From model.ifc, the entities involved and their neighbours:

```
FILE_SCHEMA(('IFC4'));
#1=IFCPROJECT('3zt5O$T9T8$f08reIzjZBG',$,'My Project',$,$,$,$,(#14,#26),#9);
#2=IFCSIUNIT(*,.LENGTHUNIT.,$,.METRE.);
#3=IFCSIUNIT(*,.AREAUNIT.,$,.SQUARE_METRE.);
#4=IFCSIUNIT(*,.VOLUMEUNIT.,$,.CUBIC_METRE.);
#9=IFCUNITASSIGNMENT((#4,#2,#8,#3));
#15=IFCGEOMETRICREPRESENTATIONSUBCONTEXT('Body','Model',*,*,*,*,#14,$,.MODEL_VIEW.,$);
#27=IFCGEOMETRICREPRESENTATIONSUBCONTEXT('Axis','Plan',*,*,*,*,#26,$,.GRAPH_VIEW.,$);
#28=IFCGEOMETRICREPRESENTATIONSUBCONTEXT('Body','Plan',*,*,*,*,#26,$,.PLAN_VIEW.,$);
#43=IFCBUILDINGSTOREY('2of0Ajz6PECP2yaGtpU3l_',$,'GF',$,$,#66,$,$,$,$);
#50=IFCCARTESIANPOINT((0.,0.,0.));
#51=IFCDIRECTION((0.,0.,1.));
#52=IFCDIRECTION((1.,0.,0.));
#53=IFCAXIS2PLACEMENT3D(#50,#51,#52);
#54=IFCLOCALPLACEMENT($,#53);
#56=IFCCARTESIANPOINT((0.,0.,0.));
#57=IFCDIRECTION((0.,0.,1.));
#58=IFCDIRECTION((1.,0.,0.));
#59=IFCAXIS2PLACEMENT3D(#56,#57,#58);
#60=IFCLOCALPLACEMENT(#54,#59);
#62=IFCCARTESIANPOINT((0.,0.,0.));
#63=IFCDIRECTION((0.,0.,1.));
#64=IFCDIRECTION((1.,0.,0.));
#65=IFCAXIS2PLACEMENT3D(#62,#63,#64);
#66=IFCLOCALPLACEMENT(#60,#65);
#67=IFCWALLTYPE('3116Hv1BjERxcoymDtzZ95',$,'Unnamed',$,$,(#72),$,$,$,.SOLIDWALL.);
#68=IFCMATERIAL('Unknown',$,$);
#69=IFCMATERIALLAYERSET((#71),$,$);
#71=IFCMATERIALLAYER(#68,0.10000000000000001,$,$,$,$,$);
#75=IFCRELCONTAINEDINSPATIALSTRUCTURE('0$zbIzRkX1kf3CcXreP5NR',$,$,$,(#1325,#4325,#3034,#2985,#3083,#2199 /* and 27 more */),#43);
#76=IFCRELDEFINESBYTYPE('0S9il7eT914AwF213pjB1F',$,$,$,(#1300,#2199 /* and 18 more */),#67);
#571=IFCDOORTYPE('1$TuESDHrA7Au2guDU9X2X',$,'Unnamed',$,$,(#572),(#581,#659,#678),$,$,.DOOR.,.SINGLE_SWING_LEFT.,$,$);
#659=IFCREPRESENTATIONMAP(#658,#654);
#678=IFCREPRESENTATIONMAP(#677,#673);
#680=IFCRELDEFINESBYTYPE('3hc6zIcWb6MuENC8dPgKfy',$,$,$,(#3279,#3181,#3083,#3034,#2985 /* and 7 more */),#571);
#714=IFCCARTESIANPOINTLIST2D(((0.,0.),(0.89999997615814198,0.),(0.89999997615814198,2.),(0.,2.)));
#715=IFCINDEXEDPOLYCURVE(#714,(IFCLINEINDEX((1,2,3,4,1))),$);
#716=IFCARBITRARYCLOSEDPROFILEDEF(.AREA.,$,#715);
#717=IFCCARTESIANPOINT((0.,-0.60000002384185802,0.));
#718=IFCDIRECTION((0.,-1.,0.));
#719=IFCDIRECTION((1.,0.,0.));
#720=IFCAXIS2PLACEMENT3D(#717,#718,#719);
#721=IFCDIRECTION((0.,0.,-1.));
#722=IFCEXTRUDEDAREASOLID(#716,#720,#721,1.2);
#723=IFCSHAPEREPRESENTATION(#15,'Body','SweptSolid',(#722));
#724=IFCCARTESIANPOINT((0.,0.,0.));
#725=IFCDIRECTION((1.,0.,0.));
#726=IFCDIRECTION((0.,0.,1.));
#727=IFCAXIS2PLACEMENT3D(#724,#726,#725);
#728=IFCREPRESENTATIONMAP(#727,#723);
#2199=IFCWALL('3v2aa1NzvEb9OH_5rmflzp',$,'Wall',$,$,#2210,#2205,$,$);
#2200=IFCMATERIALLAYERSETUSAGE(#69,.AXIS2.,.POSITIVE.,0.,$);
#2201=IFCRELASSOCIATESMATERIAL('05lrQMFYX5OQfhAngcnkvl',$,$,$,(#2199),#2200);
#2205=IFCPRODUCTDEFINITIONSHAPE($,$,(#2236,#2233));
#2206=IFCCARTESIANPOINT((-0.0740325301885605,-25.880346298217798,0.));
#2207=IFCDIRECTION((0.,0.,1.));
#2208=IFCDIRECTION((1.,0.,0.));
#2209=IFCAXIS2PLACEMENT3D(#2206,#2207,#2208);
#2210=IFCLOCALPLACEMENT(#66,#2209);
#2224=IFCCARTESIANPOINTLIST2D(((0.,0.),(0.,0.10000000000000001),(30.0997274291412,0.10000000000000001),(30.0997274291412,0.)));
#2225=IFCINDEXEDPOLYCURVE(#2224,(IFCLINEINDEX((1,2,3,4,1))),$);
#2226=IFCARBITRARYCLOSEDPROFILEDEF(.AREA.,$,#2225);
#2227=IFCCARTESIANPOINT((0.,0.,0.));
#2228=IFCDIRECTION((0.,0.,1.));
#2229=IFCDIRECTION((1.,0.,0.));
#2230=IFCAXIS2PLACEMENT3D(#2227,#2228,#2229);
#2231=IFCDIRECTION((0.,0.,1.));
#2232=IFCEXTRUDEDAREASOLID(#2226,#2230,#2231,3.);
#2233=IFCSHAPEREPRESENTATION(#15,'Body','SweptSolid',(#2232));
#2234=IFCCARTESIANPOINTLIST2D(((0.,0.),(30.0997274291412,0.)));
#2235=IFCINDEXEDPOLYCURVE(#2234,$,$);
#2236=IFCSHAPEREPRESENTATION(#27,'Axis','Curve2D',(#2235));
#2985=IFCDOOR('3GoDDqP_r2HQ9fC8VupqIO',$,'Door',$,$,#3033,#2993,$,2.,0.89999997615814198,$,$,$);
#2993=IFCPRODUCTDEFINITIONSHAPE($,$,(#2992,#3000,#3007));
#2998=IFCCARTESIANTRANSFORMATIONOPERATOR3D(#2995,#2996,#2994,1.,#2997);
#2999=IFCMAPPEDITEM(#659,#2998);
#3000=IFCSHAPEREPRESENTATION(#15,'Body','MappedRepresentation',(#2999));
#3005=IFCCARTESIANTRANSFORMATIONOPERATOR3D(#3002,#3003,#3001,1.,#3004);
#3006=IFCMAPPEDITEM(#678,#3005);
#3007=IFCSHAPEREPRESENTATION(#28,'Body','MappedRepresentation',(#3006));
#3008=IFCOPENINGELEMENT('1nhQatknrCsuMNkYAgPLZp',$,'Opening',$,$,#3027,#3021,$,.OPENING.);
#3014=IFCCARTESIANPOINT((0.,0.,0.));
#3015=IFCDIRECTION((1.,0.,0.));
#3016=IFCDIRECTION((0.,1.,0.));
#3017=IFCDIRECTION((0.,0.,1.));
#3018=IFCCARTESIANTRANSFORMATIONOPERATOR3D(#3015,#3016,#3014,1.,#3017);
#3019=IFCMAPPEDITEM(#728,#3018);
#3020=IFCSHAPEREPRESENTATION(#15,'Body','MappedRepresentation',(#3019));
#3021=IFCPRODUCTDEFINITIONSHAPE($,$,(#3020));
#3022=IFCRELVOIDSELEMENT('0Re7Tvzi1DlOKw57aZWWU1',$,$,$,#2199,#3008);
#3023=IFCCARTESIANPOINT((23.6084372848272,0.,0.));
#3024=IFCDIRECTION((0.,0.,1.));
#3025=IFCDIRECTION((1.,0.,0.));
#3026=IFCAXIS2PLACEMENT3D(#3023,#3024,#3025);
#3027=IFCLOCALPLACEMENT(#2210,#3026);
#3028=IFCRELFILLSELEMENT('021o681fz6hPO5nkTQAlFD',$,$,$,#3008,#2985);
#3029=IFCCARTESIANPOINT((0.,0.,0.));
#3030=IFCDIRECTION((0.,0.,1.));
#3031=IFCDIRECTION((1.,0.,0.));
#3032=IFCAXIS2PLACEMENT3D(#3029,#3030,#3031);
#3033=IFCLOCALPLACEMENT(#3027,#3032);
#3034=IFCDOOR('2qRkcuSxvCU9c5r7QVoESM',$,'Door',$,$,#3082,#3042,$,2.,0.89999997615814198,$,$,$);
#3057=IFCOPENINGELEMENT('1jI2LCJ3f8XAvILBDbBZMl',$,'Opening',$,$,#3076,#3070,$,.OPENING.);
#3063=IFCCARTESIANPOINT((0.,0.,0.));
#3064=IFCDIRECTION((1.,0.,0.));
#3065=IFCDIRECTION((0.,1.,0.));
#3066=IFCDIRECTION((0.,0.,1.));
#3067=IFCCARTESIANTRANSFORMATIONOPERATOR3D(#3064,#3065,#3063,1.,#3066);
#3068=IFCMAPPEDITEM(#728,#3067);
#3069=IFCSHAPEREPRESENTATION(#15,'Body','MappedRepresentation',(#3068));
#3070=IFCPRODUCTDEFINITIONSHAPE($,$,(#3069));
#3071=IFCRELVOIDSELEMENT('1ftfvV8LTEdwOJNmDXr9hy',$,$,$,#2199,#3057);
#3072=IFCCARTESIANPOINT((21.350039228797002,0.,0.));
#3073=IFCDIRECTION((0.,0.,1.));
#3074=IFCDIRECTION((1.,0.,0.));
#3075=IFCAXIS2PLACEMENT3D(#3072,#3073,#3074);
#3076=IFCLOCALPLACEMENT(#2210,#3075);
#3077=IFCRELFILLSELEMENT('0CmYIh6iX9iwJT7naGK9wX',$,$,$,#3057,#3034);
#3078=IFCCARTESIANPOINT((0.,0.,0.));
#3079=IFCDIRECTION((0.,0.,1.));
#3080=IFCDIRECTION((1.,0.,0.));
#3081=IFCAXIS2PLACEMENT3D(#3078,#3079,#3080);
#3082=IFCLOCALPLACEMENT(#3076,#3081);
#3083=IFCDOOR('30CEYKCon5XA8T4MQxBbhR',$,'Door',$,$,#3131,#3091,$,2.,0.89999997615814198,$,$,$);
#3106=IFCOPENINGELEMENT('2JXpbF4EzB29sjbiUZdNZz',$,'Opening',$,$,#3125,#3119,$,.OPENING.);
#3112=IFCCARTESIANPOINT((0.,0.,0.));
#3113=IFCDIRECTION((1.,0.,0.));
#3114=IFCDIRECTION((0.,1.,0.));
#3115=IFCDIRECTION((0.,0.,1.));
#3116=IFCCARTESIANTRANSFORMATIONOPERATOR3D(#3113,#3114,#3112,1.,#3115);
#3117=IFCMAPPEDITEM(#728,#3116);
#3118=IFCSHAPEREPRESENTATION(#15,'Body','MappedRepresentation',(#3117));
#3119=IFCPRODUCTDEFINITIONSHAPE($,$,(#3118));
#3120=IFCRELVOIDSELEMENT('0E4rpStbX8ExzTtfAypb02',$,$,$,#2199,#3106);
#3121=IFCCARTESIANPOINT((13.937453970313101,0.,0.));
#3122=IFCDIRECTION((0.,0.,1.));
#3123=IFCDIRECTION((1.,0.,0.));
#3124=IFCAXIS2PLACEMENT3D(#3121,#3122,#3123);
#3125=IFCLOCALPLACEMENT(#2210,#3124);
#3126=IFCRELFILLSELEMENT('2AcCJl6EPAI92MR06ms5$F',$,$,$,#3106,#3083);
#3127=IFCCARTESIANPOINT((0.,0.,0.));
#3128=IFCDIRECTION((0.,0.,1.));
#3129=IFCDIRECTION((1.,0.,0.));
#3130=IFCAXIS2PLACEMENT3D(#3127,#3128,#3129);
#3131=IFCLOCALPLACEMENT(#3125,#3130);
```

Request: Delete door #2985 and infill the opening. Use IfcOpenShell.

```python
import ifcopenshell
import ifcopenshell.api.feature
import ifcopenshell.api.root
import ifcopenshell.geom
import ifcopenshell.util.shape

model = ifcopenshell.open("model.ifc")
settings = ifcopenshell.geom.settings()


def volume(element):
    """Net volume in cubic metres, openings subtracted."""
    shape = ifcopenshell.geom.create_shape(settings, element)
    return ifcopenshell.util.shape.get_volume(shape.geometry)


door = model.by_guid("3GoDDqP_r2HQ9fC8VupqIO")
opening = door.FillsVoids[0].RelatingOpeningElement
wall = opening.VoidsElements[0].RelatingBuildingElement
before = volume(wall)

ifcopenshell.api.root.remove_product(model, product=door)
ifcopenshell.api.feature.remove_feature(model, feature=opening)

after = volume(wall)

print(f"wall volume {before:.3f} -> {after:.3f} m3")

model.write("model_rev.ifc")
```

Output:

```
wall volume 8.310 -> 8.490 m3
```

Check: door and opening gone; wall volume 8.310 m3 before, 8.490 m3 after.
